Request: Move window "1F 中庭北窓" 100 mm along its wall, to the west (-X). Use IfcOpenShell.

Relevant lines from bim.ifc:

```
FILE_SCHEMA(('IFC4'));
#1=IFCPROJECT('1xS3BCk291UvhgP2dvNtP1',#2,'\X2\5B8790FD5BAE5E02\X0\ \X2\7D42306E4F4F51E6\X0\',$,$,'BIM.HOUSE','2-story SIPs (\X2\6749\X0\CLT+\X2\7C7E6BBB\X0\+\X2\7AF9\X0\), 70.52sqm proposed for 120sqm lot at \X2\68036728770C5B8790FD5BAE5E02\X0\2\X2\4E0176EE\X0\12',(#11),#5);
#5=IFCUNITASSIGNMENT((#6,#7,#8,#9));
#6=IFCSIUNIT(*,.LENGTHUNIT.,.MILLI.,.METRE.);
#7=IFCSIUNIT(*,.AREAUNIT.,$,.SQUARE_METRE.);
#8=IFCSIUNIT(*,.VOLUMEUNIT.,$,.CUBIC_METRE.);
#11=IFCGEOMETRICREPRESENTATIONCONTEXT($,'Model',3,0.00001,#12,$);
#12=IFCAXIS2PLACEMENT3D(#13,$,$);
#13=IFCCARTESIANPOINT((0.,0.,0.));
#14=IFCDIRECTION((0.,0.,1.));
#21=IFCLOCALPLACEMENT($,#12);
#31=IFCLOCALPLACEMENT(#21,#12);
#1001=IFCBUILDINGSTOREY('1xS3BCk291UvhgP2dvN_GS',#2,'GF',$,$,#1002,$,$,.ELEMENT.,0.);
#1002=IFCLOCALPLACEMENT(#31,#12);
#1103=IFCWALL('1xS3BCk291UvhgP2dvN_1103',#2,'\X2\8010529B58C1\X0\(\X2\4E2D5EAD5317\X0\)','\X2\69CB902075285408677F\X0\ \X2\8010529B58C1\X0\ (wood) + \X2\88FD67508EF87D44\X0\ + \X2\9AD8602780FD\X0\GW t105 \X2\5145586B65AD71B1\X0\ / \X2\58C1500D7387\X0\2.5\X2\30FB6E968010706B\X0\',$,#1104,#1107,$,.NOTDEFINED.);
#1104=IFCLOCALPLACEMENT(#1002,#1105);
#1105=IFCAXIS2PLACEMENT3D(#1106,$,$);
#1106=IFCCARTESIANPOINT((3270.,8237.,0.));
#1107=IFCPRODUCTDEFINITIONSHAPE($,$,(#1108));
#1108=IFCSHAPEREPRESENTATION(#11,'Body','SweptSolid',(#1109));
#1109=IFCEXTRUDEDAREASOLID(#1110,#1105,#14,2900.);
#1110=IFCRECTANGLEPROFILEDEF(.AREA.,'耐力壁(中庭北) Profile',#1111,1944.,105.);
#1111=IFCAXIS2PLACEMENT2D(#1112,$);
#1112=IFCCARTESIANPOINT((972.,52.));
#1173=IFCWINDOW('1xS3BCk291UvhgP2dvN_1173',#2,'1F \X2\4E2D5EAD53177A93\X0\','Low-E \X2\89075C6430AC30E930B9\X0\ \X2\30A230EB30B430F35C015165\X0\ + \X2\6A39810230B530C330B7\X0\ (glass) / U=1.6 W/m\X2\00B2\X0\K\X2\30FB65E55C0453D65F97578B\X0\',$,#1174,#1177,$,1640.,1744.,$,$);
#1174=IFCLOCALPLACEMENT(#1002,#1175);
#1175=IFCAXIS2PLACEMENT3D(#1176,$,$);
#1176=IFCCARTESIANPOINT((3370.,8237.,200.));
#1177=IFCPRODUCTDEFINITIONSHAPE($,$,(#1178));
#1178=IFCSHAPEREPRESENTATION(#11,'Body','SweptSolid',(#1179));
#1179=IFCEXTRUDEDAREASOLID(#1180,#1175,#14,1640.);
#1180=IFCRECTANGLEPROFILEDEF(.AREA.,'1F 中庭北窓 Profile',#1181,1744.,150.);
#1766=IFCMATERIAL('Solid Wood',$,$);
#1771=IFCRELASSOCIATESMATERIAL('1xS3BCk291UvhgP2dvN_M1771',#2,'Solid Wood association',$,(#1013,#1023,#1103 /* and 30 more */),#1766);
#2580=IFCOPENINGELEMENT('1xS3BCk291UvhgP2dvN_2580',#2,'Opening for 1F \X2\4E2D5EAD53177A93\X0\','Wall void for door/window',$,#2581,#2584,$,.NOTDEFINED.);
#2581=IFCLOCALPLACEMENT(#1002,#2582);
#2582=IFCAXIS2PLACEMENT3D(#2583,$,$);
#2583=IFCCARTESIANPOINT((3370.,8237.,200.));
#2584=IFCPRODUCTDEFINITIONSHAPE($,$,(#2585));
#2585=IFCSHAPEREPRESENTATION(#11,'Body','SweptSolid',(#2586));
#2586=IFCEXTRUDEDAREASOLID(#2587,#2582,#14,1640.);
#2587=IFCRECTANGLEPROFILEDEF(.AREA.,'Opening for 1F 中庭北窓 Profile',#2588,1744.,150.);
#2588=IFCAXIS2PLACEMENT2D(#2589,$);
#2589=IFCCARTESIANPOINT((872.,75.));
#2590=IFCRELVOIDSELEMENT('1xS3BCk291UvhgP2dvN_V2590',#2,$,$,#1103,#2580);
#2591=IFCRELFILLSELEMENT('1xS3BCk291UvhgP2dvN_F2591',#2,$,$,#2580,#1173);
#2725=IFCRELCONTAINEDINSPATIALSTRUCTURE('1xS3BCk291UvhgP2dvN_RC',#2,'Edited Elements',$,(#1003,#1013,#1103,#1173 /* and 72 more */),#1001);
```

```python
import ifcopenshell
import ifcopenshell.api.geometry
import ifcopenshell.util.placement

model = ifcopenshell.open("bim.ifc")

window = model.by_id(1173)
opening = window.FillsVoids[0].RelatingOpeningElement
wall = opening.VoidsElements[0].RelatingBuildingElement

wall_matrix = ifcopenshell.util.placement.get_local_placement(wall.ObjectPlacement)
shift = wall_matrix[:3, 0] * -100.0
before = ifcopenshell.util.placement.get_local_placement(window.ObjectPlacement)[:3, 3].copy()

# The window is not placed relative to its opening, so move both.
for product in (opening, window):
    matrix = ifcopenshell.util.placement.get_local_placement(product.ObjectPlacement)
    matrix[:3, 3] += shift
    ifcopenshell.api.geometry.edit_object_placement(model, product=product, matrix=matrix, is_si=False)

after = ifcopenshell.util.placement.get_local_placement(window.ObjectPlacement)[:3, 3]
print("window moved by", (after - before).round(3) + 0.0)

model.write("bim_updated.ifc")
```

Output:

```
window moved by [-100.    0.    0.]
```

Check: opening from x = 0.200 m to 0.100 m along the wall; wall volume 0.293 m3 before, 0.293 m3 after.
